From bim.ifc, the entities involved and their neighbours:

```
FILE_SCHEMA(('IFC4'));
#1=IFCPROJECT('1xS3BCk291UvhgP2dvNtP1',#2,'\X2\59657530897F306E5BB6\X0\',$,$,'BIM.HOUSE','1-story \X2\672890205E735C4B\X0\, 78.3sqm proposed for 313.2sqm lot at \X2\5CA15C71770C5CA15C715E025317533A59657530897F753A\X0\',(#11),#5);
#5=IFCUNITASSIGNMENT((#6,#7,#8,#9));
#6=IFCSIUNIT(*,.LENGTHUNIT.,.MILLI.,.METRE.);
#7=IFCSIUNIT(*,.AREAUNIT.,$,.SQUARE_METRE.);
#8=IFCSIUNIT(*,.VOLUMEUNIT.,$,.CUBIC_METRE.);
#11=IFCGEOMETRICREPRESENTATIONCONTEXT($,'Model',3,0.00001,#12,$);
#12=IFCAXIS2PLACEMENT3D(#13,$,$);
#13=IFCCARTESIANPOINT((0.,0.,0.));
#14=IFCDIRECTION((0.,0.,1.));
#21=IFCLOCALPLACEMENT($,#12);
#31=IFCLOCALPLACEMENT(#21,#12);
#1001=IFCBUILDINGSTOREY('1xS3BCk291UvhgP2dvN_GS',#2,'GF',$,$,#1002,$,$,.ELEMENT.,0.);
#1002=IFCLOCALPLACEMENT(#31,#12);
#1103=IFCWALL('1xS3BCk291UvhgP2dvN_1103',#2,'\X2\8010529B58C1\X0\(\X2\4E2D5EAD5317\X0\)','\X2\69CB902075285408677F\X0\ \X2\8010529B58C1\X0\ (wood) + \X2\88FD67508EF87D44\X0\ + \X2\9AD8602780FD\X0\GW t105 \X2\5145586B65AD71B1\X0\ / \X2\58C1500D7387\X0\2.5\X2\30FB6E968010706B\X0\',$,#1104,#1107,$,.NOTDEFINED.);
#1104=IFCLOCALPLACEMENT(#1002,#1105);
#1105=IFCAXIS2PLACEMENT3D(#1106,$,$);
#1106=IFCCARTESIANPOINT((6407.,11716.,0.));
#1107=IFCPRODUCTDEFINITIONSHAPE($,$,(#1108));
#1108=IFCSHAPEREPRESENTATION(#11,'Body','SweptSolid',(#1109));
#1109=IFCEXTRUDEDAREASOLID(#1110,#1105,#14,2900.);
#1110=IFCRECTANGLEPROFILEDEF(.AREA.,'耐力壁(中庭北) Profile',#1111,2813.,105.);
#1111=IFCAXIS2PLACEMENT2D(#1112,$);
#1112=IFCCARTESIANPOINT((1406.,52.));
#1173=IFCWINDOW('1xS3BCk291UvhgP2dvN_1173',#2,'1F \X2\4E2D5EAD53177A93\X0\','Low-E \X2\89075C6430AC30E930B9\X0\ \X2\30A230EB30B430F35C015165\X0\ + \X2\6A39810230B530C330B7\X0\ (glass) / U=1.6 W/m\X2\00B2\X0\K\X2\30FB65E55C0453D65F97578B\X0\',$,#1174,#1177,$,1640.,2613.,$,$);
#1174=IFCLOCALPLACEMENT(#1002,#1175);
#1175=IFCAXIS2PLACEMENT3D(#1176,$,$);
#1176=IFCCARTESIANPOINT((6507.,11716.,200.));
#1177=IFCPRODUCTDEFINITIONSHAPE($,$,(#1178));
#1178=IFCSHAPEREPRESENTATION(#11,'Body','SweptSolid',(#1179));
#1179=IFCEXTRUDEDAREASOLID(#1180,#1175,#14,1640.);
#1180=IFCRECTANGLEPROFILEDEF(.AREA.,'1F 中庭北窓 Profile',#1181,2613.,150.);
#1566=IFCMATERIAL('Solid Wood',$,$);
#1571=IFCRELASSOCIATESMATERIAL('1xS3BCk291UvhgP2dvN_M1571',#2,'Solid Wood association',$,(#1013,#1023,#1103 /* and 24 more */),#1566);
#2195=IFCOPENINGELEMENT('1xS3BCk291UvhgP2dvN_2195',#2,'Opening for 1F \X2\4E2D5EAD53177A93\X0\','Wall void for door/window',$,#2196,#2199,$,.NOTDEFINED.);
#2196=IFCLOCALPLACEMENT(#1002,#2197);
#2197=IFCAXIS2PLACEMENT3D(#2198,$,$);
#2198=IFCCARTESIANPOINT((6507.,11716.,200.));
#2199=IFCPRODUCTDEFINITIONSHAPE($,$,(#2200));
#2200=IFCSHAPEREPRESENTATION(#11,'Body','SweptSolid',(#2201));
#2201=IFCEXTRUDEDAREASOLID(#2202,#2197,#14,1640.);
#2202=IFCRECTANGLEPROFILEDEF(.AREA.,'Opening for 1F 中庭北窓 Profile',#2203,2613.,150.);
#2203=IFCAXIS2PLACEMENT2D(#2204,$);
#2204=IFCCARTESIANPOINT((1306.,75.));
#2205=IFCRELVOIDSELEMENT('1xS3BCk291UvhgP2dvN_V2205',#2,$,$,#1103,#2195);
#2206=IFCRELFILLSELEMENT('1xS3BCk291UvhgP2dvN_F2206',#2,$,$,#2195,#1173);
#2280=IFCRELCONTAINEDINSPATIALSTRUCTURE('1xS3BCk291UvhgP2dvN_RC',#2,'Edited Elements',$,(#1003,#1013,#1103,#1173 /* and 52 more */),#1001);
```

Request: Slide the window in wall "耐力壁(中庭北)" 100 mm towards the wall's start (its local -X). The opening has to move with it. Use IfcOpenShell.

```python
import ifcopenshell
import ifcopenshell.api.geometry
import ifcopenshell.util.placement
import ifcopenshell.util.unit

model = ifcopenshell.open("bim.ifc")
unit_scale = ifcopenshell.util.unit.calculate_unit_scale(model)

window = model.by_id(1173)
opening = window.FillsVoids[0].RelatingOpeningElement
wall = opening.VoidsElements[0].RelatingBuildingElement

wall_matrix = ifcopenshell.util.placement.get_local_placement(wall.ObjectPlacement)
shift = wall_matrix[:3, 0] * -0.1 / unit_scale
before = ifcopenshell.util.placement.get_local_placement(window.ObjectPlacement)[:3, 3].copy()

# The window is not placed relative to its opening, so move both.
for product in (opening, window):
    matrix = ifcopenshell.util.placement.get_local_placement(product.ObjectPlacement)
    matrix[:3, 3] += shift
    ifcopenshell.api.geometry.edit_object_placement(model, product=product, matrix=matrix, is_si=False)

after = ifcopenshell.util.placement.get_local_placement(window.ObjectPlacement)[:3, 3]
print("window moved by", (after - before).round(3) + 0.0)

model.write("bim-out.ifc")
```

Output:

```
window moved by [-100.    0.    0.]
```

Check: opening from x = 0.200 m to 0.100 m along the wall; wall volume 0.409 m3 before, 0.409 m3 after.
